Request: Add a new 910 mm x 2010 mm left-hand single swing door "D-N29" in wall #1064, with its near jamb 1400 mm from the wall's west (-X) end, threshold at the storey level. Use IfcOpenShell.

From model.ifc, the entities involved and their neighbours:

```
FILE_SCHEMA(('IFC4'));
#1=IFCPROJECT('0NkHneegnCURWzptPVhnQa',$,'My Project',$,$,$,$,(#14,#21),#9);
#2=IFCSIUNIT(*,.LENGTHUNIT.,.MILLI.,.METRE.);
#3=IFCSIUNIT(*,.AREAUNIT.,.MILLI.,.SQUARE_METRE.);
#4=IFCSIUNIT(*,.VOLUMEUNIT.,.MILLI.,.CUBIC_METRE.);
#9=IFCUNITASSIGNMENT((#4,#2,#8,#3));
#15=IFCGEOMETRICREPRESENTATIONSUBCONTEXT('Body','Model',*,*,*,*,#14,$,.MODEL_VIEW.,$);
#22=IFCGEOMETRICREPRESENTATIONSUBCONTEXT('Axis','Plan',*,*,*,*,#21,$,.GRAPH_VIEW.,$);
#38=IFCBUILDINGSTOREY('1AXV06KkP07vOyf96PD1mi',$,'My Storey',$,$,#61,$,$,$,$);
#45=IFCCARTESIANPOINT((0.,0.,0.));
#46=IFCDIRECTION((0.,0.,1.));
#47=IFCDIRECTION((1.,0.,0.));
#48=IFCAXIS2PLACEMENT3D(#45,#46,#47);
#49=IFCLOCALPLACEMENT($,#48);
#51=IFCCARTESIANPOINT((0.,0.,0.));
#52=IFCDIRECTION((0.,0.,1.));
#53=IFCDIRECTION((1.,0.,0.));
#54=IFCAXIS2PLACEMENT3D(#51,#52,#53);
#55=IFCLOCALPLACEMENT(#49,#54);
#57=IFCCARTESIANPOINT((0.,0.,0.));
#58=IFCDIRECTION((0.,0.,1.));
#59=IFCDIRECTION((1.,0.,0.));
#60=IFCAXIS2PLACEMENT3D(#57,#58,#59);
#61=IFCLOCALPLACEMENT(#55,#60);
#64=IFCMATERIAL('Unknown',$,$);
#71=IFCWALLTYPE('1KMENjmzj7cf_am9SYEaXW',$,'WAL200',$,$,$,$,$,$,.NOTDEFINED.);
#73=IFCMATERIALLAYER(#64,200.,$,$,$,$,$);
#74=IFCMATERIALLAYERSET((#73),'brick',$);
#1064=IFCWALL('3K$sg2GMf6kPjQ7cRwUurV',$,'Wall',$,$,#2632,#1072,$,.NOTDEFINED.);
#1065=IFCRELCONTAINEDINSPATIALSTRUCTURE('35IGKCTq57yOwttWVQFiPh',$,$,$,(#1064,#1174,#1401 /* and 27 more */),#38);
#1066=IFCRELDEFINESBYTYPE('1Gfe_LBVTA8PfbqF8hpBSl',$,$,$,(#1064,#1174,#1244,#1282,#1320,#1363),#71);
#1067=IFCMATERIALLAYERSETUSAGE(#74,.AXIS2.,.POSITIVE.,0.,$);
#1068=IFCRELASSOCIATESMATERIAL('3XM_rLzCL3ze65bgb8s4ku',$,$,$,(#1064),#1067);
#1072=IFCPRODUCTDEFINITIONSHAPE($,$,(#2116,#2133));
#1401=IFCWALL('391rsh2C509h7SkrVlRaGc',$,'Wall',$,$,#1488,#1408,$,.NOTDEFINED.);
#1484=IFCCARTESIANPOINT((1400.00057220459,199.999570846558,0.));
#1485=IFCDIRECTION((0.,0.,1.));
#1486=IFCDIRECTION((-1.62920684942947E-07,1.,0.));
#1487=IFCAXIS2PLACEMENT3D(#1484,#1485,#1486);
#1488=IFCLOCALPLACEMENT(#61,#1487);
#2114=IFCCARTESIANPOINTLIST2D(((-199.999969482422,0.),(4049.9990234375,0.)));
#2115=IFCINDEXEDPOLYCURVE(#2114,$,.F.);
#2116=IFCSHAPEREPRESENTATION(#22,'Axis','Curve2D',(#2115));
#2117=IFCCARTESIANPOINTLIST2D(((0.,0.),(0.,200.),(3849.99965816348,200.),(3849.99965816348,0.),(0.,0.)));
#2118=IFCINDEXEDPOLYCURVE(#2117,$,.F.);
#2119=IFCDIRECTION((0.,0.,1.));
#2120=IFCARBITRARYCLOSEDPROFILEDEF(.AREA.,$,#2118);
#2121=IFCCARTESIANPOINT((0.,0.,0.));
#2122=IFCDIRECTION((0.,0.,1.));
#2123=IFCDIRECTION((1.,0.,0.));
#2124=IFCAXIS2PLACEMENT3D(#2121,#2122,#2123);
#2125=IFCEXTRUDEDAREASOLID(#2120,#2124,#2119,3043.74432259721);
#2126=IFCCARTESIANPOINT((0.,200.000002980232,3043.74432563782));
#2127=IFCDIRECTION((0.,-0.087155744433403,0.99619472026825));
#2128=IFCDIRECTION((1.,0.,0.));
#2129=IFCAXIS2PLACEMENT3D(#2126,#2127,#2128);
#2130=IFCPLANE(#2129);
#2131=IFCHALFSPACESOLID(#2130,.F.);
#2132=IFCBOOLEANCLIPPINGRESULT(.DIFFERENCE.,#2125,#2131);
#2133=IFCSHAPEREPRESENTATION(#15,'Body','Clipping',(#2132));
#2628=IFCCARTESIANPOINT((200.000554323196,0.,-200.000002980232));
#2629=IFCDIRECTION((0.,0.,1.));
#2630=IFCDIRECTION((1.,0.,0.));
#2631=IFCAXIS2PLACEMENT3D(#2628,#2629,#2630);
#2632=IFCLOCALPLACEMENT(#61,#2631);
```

```python
import numpy as np
import ifcopenshell
import ifcopenshell.api.feature
import ifcopenshell.api.geometry
import ifcopenshell.api.root
import ifcopenshell.api.spatial
import ifcopenshell.geom
import ifcopenshell.util.element
import ifcopenshell.util.placement
import ifcopenshell.util.representation
import ifcopenshell.util.shape
import ifcopenshell.util.unit

model = ifcopenshell.open("model.ifc")
unit_scale = ifcopenshell.util.unit.calculate_unit_scale(model)
settings = ifcopenshell.geom.settings()


def volume(element):
    """Net volume in cubic metres, openings subtracted."""
    shape = ifcopenshell.geom.create_shape(settings, element)
    return ifcopenshell.util.shape.get_volume(shape.geometry)


wall = model.by_id(1064)
storey = ifcopenshell.util.element.get_container(wall, ifc_class="IfcBuildingStorey")
context = ifcopenshell.util.representation.get_context(model, "Model", "Body", "MODEL_VIEW")
before = volume(wall)

width, height, from_end, sill = 0.91, 2.01, 1.4, 0.0  # metres

# The wall runs along its own X axis, and the end named is its -X end.
wall_shape = ifcopenshell.geom.create_shape(settings, wall)
x, y, z = ifcopenshell.util.shape.get_vertices(wall_shape.geometry).T
start = x.min() + from_end
face, thickness = float(y.min()), float(y.max() - y.min())
wall_matrix = ifcopenshell.util.placement.get_local_placement(wall.ObjectPlacement)
level = ifcopenshell.util.placement.get_local_placement(storey.ObjectPlacement)[2, 3]


def in_wall(x, y):
    """Placement at x, y metres in the wall's axes, at sill height."""
    matrix = wall_matrix.copy()
    matrix[:, 3] = wall_matrix @ np.array([x / unit_scale, y / unit_scale, 0.0, 1.0])
    matrix[2, 3] = level + sill / unit_scale
    return matrix


# Opening: a box that overshoots both wall faces by 50 mm.
opening = ifcopenshell.api.root.create_entity(model, ifc_class="IfcOpeningElement", predefined_type="OPENING")
box = ifcopenshell.api.geometry.add_wall_representation(
    model, context=context, length=width, height=height, thickness=thickness + 0.1
)
ifcopenshell.api.geometry.assign_representation(model, product=opening, representation=box)
ifcopenshell.api.geometry.edit_object_placement(model, product=opening, matrix=in_wall(start, face - 0.05), is_si=False)
ifcopenshell.api.feature.add_feature(model, feature=opening, element=wall)

door = ifcopenshell.api.root.create_entity(model, ifc_class="IfcDoor", name="D-N29", predefined_type="DOOR")
door.OverallWidth, door.OverallHeight = width / unit_scale, height / unit_scale
door.OperationType = "SINGLE_SWING_LEFT"
body = ifcopenshell.api.geometry.add_door_representation(
    model,
    context=context,
    overall_width=door.OverallWidth,
    overall_height=door.OverallHeight,
    operation_type="SINGLE_SWING_LEFT",
    lining_properties={"LiningDepth": thickness / unit_scale, "ThresholdDepth": thickness / unit_scale},
)
ifcopenshell.api.geometry.assign_representation(model, product=door, representation=body)
ifcopenshell.api.spatial.assign_container(model, products=[door], relating_structure=storey)
ifcopenshell.api.feature.add_filling(model, opening=opening, element=door)

# The lining spans the wall, so the door starts at the wall face.
ifcopenshell.api.geometry.edit_object_placement(model, product=door, matrix=in_wall(start, face), is_si=False)

after = volume(wall)

print(f"wall volume {before:.3f} -> {after:.3f} m3")

model.write("model_rev.ifc")
```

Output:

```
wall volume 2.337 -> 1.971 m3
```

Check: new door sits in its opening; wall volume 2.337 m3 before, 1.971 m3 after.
